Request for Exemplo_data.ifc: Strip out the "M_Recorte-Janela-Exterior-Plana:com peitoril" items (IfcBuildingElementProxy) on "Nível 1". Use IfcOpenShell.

First a look at what the model holds.

```python
import ifcopenshell
import ifcopenshell.util.element

model = ifcopenshell.open("Exemplo_data.ifc")
print(model.schema)
storey = next(s for s in model.by_type("IfcBuildingStorey") if s.Name == "Nível 1")
proxies = [e for e in ifcopenshell.util.element.get_decomposition(storey) if e.is_a("IfcBuildingElementProxy")]
seen = {}
for e in proxies:
    element_type = ifcopenshell.util.element.get_type(e)
    name = element_type.Name if element_type not in (None, e) else None
    seen[name] = seen.get(name, 0) + 1
for name, count in sorted(seen.items(), key=str):
    print(count, "x", name)
```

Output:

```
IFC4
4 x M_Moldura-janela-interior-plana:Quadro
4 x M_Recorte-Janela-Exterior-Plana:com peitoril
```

```python
import ifcopenshell
import ifcopenshell.api.root
import ifcopenshell.util.element

model = ifcopenshell.open("Exemplo_data.ifc")

storey = next(s for s in model.by_type("IfcBuildingStorey") if s.Name == "Nível 1")
proxies = [e for e in ifcopenshell.util.element.get_decomposition(storey) if e.is_a("IfcBuildingElementProxy")]
targets = [e for e in proxies if (t := ifcopenshell.util.element.get_type(e)) not in (None, e) and t.Name == "M_Recorte-Janela-Exterior-Plana:com peitoril"]

for e in targets:
    ifcopenshell.api.root.remove_product(model, product=e)
print(len(targets), "removed")

model.write("Exemplo_data-out.ifc")
```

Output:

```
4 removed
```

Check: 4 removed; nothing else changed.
